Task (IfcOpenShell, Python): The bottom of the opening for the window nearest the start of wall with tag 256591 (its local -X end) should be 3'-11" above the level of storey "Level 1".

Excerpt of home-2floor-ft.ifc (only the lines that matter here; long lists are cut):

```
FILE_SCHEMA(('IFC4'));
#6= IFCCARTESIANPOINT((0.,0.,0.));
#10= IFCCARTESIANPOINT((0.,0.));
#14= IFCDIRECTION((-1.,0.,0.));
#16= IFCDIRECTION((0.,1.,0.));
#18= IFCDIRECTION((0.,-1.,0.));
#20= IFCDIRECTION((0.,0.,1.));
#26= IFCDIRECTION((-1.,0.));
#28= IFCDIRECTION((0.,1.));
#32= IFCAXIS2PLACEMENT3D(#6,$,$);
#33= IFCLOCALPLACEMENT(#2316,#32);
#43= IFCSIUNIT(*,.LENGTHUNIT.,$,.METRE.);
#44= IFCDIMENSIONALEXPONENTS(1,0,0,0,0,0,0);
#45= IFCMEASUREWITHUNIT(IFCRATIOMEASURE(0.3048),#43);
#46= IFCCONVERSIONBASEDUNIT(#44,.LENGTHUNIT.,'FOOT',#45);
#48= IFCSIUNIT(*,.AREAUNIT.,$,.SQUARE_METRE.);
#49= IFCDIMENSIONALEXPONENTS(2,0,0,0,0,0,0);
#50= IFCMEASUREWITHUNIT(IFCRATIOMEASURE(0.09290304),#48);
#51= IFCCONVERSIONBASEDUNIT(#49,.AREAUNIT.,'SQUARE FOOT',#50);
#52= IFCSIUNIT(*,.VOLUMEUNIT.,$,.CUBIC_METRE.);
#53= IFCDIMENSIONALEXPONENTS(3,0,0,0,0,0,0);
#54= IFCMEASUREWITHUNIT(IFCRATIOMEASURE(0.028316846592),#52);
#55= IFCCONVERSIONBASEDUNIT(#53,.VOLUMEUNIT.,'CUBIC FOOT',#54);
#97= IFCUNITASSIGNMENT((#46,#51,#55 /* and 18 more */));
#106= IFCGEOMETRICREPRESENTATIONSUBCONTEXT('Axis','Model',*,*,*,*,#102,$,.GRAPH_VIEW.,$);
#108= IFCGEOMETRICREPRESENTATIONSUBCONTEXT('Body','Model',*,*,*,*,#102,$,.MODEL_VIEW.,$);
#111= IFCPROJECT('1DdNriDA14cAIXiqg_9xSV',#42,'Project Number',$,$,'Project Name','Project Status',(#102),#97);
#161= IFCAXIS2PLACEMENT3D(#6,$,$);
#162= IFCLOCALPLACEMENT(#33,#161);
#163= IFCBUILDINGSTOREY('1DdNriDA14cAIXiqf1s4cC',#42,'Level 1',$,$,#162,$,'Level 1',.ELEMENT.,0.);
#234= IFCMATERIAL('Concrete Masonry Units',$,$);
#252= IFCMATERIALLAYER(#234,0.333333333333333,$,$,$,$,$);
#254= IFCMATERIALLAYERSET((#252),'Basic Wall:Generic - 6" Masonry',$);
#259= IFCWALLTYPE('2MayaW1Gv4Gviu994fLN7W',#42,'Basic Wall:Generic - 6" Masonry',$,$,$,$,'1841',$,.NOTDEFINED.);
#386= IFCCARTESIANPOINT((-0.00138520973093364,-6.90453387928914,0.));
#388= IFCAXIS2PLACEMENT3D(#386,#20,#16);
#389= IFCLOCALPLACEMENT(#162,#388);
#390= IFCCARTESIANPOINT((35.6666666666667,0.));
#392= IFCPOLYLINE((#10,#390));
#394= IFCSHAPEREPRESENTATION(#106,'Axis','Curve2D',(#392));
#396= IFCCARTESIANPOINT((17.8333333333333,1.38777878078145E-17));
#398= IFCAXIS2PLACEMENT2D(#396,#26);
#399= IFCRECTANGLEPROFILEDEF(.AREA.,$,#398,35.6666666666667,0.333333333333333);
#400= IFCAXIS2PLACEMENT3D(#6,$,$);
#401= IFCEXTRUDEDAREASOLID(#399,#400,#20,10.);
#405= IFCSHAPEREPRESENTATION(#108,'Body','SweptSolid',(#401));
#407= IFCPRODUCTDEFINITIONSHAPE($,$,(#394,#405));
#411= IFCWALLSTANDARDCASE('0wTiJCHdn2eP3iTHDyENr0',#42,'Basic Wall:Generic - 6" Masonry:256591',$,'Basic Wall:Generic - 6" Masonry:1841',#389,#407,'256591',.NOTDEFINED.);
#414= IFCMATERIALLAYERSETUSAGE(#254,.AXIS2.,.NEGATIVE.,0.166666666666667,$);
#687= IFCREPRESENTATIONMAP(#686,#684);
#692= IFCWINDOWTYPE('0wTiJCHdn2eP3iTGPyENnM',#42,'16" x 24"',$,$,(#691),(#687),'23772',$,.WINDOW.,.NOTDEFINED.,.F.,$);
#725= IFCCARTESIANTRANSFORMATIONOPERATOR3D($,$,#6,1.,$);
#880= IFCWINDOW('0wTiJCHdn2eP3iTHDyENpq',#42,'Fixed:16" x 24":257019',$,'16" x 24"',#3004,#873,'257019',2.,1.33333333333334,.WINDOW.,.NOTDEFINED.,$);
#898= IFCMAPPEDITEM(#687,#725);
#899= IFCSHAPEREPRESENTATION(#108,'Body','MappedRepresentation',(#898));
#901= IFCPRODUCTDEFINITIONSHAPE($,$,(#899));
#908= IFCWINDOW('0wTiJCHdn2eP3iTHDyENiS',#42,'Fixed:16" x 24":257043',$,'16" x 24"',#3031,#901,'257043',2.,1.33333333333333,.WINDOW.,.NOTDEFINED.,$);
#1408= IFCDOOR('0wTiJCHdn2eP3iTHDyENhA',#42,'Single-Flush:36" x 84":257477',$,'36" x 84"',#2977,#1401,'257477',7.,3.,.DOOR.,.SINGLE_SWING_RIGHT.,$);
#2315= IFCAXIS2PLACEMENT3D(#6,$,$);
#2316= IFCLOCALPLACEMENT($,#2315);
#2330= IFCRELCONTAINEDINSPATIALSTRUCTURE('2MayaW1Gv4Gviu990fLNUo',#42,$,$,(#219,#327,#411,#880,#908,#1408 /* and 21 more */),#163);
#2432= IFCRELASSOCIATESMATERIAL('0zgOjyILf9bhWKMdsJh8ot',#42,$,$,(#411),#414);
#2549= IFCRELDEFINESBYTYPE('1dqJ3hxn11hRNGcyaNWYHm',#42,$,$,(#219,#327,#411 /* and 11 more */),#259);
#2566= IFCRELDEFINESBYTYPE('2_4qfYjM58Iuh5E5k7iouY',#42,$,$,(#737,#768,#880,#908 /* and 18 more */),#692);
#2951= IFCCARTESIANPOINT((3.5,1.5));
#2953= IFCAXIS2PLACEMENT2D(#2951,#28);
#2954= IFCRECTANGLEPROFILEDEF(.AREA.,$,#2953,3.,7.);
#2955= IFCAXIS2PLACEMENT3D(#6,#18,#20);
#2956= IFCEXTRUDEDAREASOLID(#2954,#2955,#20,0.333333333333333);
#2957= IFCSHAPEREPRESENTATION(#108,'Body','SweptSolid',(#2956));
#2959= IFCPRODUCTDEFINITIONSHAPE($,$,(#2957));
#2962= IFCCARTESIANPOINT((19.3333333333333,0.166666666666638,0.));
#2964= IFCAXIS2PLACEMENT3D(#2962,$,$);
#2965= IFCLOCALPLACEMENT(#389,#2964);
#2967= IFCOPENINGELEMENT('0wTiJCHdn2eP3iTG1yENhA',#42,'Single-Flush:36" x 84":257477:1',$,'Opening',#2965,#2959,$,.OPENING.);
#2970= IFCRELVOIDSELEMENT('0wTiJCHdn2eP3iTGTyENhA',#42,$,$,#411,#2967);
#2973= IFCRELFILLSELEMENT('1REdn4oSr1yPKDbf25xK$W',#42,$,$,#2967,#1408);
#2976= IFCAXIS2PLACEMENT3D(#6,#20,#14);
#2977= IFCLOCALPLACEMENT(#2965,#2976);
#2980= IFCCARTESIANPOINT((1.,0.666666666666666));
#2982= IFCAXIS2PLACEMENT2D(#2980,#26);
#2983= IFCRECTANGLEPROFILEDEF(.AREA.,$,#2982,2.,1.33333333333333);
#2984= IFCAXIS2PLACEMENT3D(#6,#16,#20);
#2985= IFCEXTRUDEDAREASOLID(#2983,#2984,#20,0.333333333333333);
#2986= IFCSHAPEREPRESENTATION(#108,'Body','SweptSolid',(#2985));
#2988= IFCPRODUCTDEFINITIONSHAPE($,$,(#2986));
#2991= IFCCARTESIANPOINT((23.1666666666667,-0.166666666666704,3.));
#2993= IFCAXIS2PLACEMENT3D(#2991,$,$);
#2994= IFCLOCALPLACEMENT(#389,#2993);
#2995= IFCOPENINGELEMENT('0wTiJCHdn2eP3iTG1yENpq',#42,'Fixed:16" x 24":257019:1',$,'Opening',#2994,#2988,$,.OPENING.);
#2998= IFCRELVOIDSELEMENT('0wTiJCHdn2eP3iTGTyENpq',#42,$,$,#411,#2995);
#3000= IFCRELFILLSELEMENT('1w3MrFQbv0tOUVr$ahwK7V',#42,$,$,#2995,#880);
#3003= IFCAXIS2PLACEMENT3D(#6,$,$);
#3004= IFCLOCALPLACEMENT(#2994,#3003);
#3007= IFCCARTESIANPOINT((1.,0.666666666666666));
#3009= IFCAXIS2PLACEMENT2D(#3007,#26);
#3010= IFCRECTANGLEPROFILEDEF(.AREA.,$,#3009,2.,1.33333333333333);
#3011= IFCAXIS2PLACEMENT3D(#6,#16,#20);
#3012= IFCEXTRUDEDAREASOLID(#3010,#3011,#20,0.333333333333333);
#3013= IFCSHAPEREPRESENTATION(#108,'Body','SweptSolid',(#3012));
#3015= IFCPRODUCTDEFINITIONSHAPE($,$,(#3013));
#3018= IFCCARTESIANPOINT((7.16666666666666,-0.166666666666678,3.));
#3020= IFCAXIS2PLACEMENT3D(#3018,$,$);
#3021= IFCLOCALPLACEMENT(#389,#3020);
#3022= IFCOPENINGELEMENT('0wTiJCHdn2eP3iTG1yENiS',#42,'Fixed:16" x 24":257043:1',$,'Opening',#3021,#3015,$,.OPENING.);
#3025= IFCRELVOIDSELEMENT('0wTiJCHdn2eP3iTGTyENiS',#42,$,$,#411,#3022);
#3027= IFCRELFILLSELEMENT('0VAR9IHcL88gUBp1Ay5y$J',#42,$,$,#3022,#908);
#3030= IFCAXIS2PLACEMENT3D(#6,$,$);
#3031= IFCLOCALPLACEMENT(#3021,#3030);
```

```python
import numpy as np
import ifcopenshell
import ifcopenshell.api.geometry
import ifcopenshell.geom
import ifcopenshell.util.element
import ifcopenshell.util.placement
import ifcopenshell.util.shape
import ifcopenshell.util.unit

model = ifcopenshell.open("home-2floor-ft.ifc")
unit_scale = ifcopenshell.util.unit.calculate_unit_scale(model)

window = model.by_guid("0wTiJCHdn2eP3iTHDyENiS")
opening = window.FillsVoids[0].RelatingOpeningElement
storey = ifcopenshell.util.element.get_container(window, ifc_class="IfcBuildingStorey")
level = ifcopenshell.util.placement.get_local_placement(storey.ObjectPlacement)[2, 3]

# The opening's origin need not be at the sill, so measure its lowest point.
shape = ifcopenshell.geom.create_shape(ifcopenshell.geom.settings(), opening)
bottom = ifcopenshell.util.shape.get_shape_bottom_elevation(shape, shape.geometry) / unit_scale
dz = level + 47 * 0.0254 / unit_scale - bottom

shift = np.array([0.0, 0.0, dz])
# The window is placed relative to its opening, so it follows when the opening moves.
matrix = ifcopenshell.util.placement.get_local_placement(opening.ObjectPlacement)
matrix[:3, 3] += shift
ifcopenshell.api.geometry.edit_object_placement(
    model, product=opening, matrix=matrix, is_si=False, should_transform_children=True
)

print(f"moved by {dz * unit_scale:+.3f} m")

model.write("home-2floor-ft-out.ifc")
```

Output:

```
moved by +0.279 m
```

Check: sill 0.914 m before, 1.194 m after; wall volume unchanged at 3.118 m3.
